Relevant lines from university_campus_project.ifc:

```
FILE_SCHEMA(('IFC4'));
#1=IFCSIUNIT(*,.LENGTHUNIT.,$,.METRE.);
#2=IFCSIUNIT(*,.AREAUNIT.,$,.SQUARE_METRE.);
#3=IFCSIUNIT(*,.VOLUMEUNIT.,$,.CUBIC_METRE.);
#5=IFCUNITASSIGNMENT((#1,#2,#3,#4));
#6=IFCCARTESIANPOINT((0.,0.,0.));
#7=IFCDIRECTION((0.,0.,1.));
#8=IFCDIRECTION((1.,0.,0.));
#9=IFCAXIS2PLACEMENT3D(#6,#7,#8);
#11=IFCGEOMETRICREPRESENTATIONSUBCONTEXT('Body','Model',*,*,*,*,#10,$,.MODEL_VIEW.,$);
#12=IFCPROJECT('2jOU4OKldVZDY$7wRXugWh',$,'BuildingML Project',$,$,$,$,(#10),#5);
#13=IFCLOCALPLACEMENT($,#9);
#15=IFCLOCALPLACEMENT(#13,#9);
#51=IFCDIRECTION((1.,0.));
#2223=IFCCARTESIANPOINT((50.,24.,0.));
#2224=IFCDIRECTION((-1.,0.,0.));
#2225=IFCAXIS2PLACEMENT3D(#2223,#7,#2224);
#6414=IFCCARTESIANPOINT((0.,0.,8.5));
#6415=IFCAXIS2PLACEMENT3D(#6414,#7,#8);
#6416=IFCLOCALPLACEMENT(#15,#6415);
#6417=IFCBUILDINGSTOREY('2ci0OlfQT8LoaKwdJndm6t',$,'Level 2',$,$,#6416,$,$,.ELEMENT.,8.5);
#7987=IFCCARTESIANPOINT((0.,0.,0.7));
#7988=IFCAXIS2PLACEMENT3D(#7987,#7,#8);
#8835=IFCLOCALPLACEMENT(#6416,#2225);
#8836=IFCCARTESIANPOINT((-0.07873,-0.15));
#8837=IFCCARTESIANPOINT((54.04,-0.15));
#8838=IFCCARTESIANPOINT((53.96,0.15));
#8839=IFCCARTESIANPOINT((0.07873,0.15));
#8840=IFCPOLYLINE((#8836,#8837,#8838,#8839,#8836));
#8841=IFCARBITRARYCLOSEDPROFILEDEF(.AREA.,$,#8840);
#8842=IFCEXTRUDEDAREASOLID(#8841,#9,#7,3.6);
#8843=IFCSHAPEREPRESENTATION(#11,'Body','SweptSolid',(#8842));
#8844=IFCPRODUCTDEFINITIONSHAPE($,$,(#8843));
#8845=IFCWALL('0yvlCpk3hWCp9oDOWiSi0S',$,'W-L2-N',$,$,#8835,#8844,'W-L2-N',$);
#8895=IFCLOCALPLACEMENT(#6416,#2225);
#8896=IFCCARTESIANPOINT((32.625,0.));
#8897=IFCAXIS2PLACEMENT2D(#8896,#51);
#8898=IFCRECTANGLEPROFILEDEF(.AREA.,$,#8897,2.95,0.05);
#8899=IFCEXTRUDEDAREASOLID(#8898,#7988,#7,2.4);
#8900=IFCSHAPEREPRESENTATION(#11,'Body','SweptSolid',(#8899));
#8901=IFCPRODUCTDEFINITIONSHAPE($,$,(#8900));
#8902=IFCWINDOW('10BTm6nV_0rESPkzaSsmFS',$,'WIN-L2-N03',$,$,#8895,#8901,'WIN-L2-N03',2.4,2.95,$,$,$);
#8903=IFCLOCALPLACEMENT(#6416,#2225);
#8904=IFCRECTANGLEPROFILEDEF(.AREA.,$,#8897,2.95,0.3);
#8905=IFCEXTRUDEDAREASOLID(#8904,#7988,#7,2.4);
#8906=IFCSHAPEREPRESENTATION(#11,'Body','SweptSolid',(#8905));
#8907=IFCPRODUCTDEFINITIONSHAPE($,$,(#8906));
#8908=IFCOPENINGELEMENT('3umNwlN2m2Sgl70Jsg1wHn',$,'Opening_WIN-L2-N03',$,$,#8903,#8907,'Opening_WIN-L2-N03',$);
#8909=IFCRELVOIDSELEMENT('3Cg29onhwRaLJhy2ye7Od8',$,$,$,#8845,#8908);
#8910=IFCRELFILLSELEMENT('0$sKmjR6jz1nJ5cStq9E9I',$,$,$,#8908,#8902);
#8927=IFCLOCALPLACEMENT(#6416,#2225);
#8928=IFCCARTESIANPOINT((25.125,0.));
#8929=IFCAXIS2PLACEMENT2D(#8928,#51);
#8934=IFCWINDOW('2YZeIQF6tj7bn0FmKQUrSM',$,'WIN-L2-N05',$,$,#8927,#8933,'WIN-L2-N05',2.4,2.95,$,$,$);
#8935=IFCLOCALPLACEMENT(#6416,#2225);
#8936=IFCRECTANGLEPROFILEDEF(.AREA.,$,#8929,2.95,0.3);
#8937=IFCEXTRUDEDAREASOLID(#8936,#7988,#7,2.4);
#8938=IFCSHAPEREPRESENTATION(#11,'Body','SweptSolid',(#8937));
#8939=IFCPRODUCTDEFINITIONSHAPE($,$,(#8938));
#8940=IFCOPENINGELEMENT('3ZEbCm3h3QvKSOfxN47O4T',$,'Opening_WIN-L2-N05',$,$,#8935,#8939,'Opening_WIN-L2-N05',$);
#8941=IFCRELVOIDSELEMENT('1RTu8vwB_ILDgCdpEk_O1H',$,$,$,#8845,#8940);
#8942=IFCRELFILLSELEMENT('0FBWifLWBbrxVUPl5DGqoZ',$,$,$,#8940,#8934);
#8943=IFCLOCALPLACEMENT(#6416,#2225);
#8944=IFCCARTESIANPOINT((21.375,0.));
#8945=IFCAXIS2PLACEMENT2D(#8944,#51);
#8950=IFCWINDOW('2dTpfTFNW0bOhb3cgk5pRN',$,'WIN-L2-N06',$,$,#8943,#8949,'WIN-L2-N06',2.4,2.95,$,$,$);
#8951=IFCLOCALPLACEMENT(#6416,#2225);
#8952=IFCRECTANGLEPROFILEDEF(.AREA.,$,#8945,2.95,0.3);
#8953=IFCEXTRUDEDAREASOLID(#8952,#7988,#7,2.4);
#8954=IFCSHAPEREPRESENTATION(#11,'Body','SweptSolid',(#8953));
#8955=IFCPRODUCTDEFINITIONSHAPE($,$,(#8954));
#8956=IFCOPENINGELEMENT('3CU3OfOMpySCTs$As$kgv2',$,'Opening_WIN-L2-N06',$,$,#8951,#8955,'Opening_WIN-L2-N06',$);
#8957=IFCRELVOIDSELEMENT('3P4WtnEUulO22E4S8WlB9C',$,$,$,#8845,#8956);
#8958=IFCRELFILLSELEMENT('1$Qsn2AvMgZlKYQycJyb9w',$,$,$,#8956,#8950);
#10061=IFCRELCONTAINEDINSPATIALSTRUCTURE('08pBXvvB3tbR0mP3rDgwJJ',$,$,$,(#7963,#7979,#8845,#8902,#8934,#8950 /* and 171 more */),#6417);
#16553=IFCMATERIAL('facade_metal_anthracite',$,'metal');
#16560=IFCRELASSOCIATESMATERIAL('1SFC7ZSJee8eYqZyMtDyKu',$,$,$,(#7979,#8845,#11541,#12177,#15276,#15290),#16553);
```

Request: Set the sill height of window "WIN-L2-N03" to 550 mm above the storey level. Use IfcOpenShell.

```python
import numpy as np
import ifcopenshell
import ifcopenshell.api.geometry
import ifcopenshell.geom
import ifcopenshell.util.element
import ifcopenshell.util.placement
import ifcopenshell.util.shape
import ifcopenshell.util.unit

model = ifcopenshell.open("university_campus_project.ifc")
unit_scale = ifcopenshell.util.unit.calculate_unit_scale(model)

window = model.by_id(8902)
opening = window.FillsVoids[0].RelatingOpeningElement
storey = ifcopenshell.util.element.get_container(window, ifc_class="IfcBuildingStorey")
level = ifcopenshell.util.placement.get_local_placement(storey.ObjectPlacement)[2, 3]

# The opening's origin need not be at the sill, so measure its lowest point.
shape = ifcopenshell.geom.create_shape(ifcopenshell.geom.settings(), opening)
bottom = ifcopenshell.util.shape.get_shape_bottom_elevation(shape, shape.geometry) / unit_scale
dz = level + 0.55 / unit_scale - bottom

shift = np.array([0.0, 0.0, dz])
# The window is not placed relative to its opening, so move both.
for product in (opening, window):
    matrix = ifcopenshell.util.placement.get_local_placement(product.ObjectPlacement)
    matrix[:3, 3] += shift
    ifcopenshell.api.geometry.edit_object_placement(model, product=product, matrix=matrix, is_si=False)

print(f"moved by {dz * unit_scale:+.3f} m")

model.write("university_campus_project_edited.ifc")
```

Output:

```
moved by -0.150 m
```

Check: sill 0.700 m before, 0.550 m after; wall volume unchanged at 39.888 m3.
